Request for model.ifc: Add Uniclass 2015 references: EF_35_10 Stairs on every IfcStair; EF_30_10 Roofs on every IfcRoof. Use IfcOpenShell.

First a look at what the model holds.

```python
import ifcopenshell

model = ifcopenshell.open("model.ifc")
print(model.schema)
print("classifications:", [c.Name for c in model.by_type("IfcClassification")])
for ifc_class in ("IfcDoor", "IfcRoof", "IfcStair", "IfcWall", "IfcWindow"):
    print(ifc_class, len(model.by_type(ifc_class)))
```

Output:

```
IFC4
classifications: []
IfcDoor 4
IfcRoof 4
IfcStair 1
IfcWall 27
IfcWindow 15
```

```python
import ifcopenshell
import ifcopenshell.api.classification

model = ifcopenshell.open("model.ifc")

system = ifcopenshell.api.classification.add_classification(model, classification="Uniclass 2015")

codes = {
    "IfcStair": ("EF_35_10", "Stairs"),
    "IfcRoof": ("EF_30_10", "Roofs"),
}
for ifc_class, (code, name) in codes.items():
    products = model.by_type(ifc_class)
    ifcopenshell.api.classification.add_reference(
        model, products=products, classification=system, identification=code, name=name
    )
    print(code, len(products))

model.write("model_v2.ifc")
```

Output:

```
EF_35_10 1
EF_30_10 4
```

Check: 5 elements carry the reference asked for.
